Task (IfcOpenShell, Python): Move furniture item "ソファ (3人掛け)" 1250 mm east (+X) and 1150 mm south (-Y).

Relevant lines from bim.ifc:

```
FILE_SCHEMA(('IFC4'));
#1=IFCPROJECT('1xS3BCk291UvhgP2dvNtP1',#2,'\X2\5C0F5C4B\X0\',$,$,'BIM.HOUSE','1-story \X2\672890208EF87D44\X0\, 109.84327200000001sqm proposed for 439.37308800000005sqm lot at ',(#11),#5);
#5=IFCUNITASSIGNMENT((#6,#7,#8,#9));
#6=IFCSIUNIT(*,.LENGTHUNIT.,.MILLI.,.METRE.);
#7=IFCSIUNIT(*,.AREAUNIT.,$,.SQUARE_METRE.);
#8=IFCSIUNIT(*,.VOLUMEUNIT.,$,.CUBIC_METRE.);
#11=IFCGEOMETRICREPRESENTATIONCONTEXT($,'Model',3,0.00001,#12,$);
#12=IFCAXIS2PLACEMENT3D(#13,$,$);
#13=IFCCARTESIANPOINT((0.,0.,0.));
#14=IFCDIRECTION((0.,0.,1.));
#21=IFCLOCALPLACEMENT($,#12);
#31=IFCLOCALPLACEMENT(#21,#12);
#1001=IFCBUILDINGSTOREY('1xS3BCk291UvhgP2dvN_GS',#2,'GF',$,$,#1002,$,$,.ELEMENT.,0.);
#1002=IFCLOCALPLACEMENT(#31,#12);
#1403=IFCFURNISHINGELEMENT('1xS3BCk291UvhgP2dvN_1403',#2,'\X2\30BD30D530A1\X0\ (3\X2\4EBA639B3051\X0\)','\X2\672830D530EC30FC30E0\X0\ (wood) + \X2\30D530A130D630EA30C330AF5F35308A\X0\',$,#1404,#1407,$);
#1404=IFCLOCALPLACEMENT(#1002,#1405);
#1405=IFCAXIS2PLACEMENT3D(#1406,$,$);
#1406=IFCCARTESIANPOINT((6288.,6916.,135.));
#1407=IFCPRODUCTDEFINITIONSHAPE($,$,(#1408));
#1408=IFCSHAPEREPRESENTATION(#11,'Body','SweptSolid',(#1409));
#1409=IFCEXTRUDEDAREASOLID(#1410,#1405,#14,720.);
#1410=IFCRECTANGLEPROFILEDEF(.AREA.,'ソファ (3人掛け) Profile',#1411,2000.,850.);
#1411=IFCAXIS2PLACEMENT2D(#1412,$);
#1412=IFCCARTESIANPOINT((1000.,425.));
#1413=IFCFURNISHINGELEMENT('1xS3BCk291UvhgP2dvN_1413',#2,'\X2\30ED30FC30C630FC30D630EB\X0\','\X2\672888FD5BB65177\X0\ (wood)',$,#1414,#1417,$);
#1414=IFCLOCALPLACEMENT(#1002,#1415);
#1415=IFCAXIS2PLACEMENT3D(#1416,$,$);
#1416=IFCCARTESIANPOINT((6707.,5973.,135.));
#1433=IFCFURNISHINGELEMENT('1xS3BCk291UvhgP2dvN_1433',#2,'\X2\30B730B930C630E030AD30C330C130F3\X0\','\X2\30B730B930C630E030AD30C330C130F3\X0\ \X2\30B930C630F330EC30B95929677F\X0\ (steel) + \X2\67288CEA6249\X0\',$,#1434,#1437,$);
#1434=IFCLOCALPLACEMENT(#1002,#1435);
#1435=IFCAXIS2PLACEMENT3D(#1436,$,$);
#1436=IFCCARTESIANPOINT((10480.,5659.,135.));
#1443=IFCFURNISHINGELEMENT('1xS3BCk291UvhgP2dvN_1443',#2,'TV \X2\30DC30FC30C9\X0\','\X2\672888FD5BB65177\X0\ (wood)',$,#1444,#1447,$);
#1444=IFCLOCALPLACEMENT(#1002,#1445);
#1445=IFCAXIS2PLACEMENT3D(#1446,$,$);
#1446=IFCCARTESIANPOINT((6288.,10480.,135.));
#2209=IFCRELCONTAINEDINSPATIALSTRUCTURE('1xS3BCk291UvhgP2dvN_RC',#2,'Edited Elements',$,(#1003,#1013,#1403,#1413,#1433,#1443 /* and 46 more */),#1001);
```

```python
import ifcopenshell
import ifcopenshell.api.geometry
import ifcopenshell.util.placement

model = ifcopenshell.open("bim.ifc")

item = model.by_id(1403)
matrix = ifcopenshell.util.placement.get_local_placement(item.ObjectPlacement)
matrix[0, 3] += 1250.0
matrix[1, 3] -= 1150.0
ifcopenshell.api.geometry.edit_object_placement(model, product=item, matrix=matrix, is_si=False)

print(ifcopenshell.util.placement.get_local_placement(item.ObjectPlacement).round(3) + 0.0)

model.write("bim_rev.ifc")
```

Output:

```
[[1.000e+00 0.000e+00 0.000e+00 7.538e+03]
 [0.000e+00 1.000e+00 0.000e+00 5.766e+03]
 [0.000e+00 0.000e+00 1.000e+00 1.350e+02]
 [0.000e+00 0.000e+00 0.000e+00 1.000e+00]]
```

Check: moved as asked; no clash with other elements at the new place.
